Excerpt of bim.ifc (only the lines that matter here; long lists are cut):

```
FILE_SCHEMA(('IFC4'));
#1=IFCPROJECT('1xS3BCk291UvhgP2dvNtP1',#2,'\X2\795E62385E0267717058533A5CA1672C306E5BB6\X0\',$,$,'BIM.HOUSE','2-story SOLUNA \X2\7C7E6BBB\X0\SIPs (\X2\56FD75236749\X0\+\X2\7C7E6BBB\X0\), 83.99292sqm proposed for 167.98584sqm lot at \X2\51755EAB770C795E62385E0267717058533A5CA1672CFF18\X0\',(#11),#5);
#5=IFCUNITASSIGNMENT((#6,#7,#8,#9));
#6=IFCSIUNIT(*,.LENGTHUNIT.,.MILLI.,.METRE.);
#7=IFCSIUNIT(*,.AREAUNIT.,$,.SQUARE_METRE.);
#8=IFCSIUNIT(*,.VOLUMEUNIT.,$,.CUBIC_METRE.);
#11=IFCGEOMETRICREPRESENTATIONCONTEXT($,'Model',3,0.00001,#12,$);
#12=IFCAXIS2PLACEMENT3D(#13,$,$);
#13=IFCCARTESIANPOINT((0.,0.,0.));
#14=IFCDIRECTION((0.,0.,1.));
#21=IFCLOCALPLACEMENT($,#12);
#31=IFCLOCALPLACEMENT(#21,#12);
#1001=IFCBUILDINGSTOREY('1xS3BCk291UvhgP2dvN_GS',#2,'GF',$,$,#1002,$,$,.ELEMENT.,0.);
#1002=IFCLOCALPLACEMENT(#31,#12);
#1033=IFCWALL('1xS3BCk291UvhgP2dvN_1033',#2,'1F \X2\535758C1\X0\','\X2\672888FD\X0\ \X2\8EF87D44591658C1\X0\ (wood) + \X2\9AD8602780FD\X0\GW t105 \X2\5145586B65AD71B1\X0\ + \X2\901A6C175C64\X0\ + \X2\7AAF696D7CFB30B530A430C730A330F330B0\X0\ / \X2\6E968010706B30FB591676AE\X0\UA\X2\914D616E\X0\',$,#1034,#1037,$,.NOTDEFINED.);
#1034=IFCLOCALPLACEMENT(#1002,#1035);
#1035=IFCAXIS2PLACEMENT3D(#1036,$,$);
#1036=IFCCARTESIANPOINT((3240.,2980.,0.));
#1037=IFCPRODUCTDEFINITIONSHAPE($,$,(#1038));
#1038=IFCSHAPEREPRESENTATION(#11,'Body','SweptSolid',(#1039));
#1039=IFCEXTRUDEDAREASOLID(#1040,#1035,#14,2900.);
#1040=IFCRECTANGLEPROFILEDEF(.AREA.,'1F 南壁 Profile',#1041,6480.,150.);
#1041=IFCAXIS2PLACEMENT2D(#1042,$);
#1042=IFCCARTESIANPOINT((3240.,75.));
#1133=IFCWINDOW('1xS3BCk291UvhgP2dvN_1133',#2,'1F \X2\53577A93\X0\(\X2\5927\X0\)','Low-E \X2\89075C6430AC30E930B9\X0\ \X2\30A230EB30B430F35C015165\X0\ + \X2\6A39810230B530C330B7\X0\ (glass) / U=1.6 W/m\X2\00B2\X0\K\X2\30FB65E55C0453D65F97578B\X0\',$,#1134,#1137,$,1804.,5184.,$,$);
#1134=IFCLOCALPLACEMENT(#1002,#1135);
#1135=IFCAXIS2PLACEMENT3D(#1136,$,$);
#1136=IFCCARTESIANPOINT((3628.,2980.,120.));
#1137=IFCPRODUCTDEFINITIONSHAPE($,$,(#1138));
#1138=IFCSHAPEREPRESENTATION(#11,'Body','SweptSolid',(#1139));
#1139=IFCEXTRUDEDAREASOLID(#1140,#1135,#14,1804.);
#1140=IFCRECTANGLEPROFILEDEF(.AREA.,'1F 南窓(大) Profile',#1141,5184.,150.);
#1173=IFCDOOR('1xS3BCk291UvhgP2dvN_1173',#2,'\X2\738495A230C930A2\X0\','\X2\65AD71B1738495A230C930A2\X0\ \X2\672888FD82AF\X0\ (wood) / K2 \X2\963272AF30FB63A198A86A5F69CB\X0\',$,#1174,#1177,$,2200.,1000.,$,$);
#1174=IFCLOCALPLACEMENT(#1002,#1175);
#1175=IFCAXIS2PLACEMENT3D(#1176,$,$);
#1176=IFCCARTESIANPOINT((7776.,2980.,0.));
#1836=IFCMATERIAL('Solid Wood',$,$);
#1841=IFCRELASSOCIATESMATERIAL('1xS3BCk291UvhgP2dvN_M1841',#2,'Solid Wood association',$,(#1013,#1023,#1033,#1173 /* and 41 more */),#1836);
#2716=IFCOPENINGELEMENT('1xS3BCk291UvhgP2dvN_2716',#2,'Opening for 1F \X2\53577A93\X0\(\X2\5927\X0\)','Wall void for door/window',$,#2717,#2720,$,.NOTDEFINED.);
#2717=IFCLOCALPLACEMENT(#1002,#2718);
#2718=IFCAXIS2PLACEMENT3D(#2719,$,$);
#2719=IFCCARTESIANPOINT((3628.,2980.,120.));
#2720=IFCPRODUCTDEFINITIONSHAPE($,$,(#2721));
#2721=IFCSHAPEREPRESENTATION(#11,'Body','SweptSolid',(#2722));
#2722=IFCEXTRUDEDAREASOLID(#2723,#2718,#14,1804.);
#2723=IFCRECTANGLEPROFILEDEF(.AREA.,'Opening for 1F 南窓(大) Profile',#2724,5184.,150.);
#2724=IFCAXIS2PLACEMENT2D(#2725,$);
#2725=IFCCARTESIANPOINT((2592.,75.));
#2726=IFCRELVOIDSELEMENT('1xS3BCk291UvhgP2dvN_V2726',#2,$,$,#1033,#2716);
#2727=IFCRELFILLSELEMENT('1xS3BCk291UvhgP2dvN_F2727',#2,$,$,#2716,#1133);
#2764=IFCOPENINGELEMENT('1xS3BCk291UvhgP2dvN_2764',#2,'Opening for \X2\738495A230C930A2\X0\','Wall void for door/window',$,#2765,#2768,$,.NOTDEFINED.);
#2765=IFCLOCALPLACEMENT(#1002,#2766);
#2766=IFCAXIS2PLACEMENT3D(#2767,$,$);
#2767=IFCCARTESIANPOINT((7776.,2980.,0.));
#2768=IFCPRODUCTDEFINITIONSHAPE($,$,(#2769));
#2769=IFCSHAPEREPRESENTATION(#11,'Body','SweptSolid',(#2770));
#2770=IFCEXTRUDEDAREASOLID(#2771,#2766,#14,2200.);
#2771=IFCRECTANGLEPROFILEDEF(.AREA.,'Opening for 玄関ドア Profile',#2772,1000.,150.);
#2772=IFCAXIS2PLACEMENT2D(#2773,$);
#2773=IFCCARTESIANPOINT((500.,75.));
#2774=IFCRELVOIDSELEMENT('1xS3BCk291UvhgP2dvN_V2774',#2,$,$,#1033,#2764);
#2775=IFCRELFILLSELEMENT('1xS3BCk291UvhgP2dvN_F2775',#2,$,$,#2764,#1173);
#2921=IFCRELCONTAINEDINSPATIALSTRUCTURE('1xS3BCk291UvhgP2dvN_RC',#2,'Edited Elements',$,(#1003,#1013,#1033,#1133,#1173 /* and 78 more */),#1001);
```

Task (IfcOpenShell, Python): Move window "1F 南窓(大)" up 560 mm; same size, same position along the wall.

```python
import numpy as np
import ifcopenshell
import ifcopenshell.api.geometry
import ifcopenshell.util.placement
import ifcopenshell.util.unit

model = ifcopenshell.open("bim.ifc")
unit_scale = ifcopenshell.util.unit.calculate_unit_scale(model)

window = model.by_id(1133)
opening = window.FillsVoids[0].RelatingOpeningElement
dz = 560.0

shift = np.array([0.0, 0.0, dz])
# The window is not placed relative to its opening, so move both.
for product in (opening, window):
    matrix = ifcopenshell.util.placement.get_local_placement(product.ObjectPlacement)
    matrix[:3, 3] += shift
    ifcopenshell.api.geometry.edit_object_placement(model, product=product, matrix=matrix, is_si=False)

print(f"moved by {dz * unit_scale:+.3f} m")

model.write("bim_updated.ifc")
```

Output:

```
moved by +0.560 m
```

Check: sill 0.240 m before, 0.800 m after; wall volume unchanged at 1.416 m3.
